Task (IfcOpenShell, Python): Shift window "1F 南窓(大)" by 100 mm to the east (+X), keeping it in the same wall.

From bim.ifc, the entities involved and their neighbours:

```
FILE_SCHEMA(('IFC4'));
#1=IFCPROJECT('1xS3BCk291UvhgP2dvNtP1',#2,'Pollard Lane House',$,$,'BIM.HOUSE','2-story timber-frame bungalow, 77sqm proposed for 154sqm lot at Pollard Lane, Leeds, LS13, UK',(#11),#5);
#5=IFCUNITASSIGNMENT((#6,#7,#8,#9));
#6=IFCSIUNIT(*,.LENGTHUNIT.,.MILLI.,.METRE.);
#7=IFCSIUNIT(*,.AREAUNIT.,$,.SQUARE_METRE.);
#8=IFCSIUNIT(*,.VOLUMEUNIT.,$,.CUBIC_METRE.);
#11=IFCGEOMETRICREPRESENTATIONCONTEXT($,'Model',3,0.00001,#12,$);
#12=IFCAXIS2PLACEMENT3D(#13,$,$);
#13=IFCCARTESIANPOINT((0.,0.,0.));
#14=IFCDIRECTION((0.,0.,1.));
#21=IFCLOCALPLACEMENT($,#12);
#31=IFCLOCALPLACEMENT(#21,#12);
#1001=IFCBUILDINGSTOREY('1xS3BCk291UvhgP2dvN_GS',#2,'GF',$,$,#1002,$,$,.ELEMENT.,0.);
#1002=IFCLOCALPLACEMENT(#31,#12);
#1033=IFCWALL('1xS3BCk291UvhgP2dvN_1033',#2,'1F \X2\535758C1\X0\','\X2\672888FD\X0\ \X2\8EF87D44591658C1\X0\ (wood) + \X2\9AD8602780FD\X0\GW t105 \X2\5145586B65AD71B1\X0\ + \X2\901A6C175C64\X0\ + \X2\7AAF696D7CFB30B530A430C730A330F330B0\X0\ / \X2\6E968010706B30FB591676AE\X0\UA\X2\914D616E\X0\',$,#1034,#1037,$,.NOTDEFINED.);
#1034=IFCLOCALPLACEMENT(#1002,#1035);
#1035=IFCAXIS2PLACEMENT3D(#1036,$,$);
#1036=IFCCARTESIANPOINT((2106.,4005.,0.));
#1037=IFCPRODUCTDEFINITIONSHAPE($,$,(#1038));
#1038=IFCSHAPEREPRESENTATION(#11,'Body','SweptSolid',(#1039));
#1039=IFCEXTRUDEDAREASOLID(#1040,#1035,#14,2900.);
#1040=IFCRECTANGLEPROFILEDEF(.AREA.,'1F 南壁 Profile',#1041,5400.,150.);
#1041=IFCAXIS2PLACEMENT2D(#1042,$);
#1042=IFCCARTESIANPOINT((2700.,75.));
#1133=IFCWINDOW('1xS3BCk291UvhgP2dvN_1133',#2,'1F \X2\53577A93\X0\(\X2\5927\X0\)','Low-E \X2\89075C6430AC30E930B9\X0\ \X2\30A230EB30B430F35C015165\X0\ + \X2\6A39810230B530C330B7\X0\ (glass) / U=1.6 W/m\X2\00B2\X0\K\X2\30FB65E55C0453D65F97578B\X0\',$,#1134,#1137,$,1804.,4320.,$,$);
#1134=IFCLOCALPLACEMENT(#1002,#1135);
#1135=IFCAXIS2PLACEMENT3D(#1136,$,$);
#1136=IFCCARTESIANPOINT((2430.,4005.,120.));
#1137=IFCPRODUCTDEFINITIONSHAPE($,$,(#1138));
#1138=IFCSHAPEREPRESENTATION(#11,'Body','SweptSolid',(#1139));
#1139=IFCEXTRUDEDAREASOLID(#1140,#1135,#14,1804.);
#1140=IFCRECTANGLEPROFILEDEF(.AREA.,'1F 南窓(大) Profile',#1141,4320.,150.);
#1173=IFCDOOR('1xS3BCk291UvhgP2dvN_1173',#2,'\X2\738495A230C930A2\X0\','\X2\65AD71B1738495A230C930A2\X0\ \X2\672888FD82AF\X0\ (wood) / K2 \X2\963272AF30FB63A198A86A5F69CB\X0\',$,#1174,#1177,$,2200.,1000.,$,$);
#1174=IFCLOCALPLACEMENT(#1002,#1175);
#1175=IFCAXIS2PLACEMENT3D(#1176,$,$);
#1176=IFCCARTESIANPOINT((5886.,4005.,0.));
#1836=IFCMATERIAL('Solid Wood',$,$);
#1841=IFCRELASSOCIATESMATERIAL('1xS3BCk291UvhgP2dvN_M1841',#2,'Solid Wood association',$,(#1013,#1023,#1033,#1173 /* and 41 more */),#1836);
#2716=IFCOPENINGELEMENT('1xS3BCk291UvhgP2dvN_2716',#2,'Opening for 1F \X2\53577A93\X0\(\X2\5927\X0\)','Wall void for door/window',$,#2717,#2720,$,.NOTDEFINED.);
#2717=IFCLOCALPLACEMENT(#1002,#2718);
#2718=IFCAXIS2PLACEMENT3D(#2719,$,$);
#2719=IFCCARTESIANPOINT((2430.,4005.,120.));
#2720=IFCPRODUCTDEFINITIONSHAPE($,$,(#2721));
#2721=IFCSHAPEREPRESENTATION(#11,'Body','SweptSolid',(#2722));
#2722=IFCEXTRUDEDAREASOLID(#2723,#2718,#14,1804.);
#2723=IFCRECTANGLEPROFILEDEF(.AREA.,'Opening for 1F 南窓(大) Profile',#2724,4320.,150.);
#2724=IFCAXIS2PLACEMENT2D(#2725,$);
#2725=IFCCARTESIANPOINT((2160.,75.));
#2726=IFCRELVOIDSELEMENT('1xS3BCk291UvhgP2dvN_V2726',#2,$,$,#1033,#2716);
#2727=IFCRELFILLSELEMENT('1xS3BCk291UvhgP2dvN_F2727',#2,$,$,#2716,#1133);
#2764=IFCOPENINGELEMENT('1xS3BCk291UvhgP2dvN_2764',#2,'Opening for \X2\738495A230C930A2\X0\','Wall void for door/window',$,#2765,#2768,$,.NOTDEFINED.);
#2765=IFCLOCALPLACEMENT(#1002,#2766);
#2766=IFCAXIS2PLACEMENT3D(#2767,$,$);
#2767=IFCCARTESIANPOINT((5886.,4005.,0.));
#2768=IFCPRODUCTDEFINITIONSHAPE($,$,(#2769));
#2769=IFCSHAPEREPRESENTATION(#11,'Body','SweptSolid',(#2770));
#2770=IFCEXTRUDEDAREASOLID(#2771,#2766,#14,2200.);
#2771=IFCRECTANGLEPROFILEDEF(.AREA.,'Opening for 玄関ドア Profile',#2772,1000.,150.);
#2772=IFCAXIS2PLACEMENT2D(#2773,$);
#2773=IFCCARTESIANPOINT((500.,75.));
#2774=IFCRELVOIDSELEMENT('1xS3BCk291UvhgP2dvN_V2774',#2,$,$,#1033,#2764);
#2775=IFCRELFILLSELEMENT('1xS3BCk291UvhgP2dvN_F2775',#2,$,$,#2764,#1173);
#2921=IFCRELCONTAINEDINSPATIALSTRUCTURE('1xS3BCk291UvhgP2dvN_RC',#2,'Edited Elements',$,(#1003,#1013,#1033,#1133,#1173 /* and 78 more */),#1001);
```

```python
import ifcopenshell
import ifcopenshell.api.geometry
import ifcopenshell.util.placement
import ifcopenshell.util.unit

model = ifcopenshell.open("bim.ifc")
unit_scale = ifcopenshell.util.unit.calculate_unit_scale(model)

window = model.by_guid("1xS3BCk291UvhgP2dvN_1133")
opening = window.FillsVoids[0].RelatingOpeningElement
wall = opening.VoidsElements[0].RelatingBuildingElement

wall_matrix = ifcopenshell.util.placement.get_local_placement(wall.ObjectPlacement)
shift = wall_matrix[:3, 0] * 0.1 / unit_scale
before = ifcopenshell.util.placement.get_local_placement(window.ObjectPlacement)[:3, 3].copy()

# The window is not placed relative to its opening, so move both.
for product in (opening, window):
    matrix = ifcopenshell.util.placement.get_local_placement(product.ObjectPlacement)
    matrix[:3, 3] += shift
    ifcopenshell.api.geometry.edit_object_placement(model, product=product, matrix=matrix, is_si=False)

after = ifcopenshell.util.placement.get_local_placement(window.ObjectPlacement)[:3, 3]
print("window moved by", (after - before).round(3) + 0.0)

model.write("bim-out.ifc")
```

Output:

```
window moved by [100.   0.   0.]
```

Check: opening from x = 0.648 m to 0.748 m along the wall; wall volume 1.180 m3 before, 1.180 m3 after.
